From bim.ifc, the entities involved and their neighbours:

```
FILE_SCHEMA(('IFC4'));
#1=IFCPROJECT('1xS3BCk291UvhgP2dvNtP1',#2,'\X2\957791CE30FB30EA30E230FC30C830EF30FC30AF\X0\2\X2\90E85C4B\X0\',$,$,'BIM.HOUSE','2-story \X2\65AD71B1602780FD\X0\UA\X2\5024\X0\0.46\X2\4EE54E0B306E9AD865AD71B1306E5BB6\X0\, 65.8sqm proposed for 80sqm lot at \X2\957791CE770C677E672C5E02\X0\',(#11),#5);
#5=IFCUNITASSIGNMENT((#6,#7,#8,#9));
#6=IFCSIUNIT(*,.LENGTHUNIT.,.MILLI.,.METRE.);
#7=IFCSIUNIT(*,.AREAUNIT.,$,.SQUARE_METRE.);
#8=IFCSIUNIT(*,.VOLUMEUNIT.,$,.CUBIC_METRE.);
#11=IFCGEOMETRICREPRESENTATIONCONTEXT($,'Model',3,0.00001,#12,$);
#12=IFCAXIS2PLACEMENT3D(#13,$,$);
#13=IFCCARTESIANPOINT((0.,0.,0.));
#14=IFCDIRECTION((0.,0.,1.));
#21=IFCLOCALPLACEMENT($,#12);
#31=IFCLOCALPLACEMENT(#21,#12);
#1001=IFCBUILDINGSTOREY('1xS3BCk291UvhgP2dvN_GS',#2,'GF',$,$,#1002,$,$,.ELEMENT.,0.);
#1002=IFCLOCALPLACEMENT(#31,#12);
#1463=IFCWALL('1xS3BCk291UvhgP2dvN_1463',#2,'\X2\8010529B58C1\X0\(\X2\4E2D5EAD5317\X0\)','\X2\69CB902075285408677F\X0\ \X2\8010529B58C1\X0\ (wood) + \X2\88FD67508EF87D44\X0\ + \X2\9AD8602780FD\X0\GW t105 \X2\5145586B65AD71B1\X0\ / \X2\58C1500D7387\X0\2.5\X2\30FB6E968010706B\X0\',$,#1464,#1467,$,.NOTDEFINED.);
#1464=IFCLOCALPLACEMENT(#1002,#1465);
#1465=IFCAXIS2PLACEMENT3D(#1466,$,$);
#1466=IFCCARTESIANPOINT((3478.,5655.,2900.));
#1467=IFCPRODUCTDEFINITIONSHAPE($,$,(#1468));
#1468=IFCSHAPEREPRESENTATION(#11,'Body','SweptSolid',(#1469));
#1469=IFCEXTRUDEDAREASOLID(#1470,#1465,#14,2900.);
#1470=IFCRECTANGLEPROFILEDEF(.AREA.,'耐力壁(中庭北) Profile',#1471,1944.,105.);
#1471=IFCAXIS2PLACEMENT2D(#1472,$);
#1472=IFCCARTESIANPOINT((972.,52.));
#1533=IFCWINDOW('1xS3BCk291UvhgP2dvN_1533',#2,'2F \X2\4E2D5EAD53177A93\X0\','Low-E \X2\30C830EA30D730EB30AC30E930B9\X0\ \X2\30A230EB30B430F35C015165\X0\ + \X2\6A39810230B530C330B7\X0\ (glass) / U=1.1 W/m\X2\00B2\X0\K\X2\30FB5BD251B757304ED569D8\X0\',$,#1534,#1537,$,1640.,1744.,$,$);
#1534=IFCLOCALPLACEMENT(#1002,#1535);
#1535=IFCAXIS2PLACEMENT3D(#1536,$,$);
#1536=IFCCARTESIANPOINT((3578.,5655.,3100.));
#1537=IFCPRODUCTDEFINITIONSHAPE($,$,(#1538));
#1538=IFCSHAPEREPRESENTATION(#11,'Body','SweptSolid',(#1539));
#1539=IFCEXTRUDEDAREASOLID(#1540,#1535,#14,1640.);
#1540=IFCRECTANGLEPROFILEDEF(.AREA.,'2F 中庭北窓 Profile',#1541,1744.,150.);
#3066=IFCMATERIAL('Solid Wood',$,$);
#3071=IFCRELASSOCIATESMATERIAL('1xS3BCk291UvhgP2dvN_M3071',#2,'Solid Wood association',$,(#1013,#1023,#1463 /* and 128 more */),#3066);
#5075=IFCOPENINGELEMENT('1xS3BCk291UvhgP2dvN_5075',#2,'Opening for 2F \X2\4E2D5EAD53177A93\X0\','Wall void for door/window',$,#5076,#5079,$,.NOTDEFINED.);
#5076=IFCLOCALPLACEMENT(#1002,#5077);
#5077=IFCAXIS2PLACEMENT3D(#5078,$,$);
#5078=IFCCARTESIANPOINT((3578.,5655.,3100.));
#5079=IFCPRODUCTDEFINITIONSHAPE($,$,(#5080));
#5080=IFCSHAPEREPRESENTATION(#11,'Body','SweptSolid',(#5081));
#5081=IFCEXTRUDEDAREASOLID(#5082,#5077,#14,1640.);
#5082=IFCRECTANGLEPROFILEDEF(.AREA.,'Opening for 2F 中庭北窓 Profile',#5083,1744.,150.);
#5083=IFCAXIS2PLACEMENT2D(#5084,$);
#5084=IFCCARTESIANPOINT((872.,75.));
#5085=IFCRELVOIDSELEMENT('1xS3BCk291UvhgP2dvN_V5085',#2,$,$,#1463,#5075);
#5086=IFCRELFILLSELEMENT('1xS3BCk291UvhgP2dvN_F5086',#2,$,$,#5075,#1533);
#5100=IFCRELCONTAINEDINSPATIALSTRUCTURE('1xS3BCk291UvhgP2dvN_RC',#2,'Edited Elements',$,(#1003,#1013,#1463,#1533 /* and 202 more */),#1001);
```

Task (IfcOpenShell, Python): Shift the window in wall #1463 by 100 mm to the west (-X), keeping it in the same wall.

```python
import ifcopenshell
import ifcopenshell.api.geometry
import ifcopenshell.util.placement
import ifcopenshell.util.unit

model = ifcopenshell.open("bim.ifc")
unit_scale = ifcopenshell.util.unit.calculate_unit_scale(model)

window = model.by_id(1533)
opening = window.FillsVoids[0].RelatingOpeningElement
wall = opening.VoidsElements[0].RelatingBuildingElement

wall_matrix = ifcopenshell.util.placement.get_local_placement(wall.ObjectPlacement)
shift = wall_matrix[:3, 0] * -0.1 / unit_scale
before = ifcopenshell.util.placement.get_local_placement(window.ObjectPlacement)[:3, 3].copy()

# The window is not placed relative to its opening, so move both.
for product in (opening, window):
    matrix = ifcopenshell.util.placement.get_local_placement(product.ObjectPlacement)
    matrix[:3, 3] += shift
    ifcopenshell.api.geometry.edit_object_placement(model, product=product, matrix=matrix, is_si=False)

after = ifcopenshell.util.placement.get_local_placement(window.ObjectPlacement)[:3, 3]
print("window moved by", (after - before).round(3) + 0.0)

model.write("bim-out.ifc")
```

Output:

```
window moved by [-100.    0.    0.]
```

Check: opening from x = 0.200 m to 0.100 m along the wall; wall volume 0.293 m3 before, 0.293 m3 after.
